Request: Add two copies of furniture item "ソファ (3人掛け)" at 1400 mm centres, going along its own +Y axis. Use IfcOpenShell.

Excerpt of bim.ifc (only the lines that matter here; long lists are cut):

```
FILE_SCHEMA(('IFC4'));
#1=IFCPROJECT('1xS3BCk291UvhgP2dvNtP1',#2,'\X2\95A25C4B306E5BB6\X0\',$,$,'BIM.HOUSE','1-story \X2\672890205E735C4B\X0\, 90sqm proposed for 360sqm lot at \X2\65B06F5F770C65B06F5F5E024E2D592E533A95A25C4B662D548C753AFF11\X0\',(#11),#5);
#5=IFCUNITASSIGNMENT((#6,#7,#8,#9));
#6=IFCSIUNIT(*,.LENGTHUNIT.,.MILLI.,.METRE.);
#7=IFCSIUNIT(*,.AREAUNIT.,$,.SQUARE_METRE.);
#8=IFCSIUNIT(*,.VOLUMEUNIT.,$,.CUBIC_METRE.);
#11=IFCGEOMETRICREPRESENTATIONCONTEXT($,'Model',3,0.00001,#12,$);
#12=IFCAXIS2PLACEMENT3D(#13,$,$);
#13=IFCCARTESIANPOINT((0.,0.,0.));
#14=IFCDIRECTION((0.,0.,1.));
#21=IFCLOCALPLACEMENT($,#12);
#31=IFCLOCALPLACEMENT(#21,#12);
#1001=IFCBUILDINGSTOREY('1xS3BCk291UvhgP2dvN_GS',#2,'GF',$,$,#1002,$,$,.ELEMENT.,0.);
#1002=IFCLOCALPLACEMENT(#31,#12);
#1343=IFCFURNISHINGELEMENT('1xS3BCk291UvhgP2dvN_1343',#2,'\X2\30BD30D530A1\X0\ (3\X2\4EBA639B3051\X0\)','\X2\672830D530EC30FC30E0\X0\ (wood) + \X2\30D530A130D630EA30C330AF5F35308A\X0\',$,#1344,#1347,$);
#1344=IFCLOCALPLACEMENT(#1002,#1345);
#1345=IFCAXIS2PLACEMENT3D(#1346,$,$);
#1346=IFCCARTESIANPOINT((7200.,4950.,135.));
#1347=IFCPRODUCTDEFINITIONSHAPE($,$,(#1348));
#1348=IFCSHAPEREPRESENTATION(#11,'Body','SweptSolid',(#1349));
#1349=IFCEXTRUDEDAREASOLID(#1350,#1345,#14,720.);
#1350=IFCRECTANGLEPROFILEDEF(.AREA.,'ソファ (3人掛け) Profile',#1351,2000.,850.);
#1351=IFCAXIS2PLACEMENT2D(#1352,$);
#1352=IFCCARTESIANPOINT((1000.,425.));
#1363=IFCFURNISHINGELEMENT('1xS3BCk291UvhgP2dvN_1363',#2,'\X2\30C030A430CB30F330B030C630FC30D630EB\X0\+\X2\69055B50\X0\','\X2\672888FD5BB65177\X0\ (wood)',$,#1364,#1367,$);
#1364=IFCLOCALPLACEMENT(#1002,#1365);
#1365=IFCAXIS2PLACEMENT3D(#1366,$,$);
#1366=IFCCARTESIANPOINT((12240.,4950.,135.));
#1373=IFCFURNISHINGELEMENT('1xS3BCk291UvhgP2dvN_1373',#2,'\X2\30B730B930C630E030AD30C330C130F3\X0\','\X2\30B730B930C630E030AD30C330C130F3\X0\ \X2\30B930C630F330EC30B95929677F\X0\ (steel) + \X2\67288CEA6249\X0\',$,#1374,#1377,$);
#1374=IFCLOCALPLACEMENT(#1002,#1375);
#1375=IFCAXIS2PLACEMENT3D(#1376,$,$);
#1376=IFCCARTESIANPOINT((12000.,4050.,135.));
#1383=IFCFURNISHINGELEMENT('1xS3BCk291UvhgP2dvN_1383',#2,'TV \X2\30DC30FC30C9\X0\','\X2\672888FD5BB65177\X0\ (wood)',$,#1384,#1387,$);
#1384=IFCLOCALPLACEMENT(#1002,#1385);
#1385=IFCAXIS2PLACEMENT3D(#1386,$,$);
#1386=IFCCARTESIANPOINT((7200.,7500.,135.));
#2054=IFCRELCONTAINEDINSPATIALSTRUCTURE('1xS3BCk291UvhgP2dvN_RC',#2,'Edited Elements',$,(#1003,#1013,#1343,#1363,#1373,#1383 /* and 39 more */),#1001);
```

```python
import ifcopenshell
import ifcopenshell.api.geometry
import ifcopenshell.api.root
import ifcopenshell.util.element
import ifcopenshell.util.placement
import ifcopenshell.util.unit

model = ifcopenshell.open("bim.ifc")
unit_scale = ifcopenshell.util.unit.calculate_unit_scale(model)


def reuse_history(source, copy):
    """copy_class also copies each property set's owner history, people and application; keep the originals."""
    for rel in copy.IsDefinedBy:
        if rel.is_a("IfcRelDefinesByProperties") and (history := rel.RelatingPropertyDefinition.OwnerHistory):
            rel.RelatingPropertyDefinition.OwnerHistory = source.OwnerHistory
            ifcopenshell.util.element.remove_deep2(model, history)


source = model.by_id(1343)
base = ifcopenshell.util.placement.get_local_placement(source.ObjectPlacement)
step = base[:3, 1] * 1.4 / unit_scale

for i in range(1, 3):
    copy = ifcopenshell.api.root.copy_class(model, product=source)
    copy.Representation = ifcopenshell.util.element.copy_deep(
        model, source.Representation, exclude=["IfcGeometricRepresentationContext", "IfcRepresentationMap"]
    )
    reuse_history(source, copy)
    matrix = base.copy()
    matrix[:3, 3] += i * step
    print("added at", matrix[:3, 3].round(3) + 0.0)
    ifcopenshell.api.geometry.edit_object_placement(model, product=copy, matrix=matrix, is_si=False)

model.write("bim-out.ifc")
```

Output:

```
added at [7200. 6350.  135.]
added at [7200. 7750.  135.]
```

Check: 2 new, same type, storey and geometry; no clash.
